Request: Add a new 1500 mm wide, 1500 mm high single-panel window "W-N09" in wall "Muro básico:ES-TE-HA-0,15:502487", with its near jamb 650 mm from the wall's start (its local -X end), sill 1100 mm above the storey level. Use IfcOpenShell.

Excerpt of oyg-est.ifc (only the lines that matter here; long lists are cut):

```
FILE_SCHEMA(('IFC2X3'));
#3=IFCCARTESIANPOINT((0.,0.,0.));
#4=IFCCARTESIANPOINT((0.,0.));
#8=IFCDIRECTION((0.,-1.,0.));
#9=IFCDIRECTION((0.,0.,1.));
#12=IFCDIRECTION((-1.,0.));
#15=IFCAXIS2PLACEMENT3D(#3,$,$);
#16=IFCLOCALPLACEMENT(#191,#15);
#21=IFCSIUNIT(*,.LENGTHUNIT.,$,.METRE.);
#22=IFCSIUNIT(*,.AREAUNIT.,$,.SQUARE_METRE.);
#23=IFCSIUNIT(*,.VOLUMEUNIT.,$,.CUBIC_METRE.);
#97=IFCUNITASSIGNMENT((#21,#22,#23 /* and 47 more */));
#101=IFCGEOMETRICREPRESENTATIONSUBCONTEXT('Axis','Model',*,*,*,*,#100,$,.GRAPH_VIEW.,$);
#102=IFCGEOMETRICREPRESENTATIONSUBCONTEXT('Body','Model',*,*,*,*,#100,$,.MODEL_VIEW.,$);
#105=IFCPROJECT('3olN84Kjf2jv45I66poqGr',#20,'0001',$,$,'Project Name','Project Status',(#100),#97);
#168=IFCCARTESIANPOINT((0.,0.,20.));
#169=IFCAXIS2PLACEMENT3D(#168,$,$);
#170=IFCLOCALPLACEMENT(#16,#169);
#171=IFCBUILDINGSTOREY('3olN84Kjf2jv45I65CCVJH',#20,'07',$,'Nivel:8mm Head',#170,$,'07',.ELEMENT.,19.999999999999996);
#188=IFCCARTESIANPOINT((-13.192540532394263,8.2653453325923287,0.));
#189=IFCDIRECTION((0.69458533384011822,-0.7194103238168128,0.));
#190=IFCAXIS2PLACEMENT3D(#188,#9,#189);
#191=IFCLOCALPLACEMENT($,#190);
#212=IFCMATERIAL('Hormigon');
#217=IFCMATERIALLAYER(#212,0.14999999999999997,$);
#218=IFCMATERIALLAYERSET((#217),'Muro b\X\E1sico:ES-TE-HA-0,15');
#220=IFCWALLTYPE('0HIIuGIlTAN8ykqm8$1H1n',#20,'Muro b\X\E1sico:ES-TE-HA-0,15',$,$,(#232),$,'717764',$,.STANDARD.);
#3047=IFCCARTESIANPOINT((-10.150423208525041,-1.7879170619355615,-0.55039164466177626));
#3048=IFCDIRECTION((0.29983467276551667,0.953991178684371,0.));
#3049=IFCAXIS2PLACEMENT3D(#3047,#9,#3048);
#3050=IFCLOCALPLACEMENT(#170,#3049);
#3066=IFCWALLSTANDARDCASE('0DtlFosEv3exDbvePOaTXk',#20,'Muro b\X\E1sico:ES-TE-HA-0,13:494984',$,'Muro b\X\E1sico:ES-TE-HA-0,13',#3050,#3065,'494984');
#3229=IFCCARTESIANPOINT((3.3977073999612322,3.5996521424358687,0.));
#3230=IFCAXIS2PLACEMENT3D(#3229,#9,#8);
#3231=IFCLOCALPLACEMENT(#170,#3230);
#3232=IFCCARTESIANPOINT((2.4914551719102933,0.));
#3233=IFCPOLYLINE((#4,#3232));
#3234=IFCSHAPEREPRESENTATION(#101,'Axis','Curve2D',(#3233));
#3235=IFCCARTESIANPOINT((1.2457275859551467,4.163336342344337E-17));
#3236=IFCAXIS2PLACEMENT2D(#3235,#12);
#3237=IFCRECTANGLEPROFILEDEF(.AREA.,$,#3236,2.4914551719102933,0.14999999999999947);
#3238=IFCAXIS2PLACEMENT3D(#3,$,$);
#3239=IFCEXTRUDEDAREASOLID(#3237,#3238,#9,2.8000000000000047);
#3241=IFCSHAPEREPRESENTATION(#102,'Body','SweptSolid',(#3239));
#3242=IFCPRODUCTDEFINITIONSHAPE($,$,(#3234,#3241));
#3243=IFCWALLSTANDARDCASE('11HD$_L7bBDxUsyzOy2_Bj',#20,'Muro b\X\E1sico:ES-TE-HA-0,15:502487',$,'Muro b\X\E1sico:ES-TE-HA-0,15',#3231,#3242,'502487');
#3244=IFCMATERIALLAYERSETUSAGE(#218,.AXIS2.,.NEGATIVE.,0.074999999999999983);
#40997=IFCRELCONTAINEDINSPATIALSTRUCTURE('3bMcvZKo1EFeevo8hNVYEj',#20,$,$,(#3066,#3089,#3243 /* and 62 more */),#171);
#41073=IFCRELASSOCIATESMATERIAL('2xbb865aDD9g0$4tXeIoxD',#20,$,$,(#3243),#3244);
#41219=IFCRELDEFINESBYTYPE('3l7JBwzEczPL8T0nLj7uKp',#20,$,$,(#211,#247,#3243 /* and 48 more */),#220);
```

```python
import numpy as np
import ifcopenshell
import ifcopenshell.api.feature
import ifcopenshell.api.geometry
import ifcopenshell.api.root
import ifcopenshell.api.spatial
import ifcopenshell.api.type
import ifcopenshell.geom
import ifcopenshell.util.element
import ifcopenshell.util.placement
import ifcopenshell.util.representation
import ifcopenshell.util.shape
import ifcopenshell.util.unit

model = ifcopenshell.open("oyg-est.ifc")
unit_scale = ifcopenshell.util.unit.calculate_unit_scale(model)
settings = ifcopenshell.geom.settings()


def volume(element):
    """Net volume in cubic metres, openings subtracted."""
    shape = ifcopenshell.geom.create_shape(settings, element)
    return ifcopenshell.util.shape.get_volume(shape.geometry)


wall = model.by_guid("11HD$_L7bBDxUsyzOy2_Bj")
storey = ifcopenshell.util.element.get_container(wall, ifc_class="IfcBuildingStorey")
context = ifcopenshell.util.representation.get_context(model, "Model", "Body", "MODEL_VIEW")
before = volume(wall)

width, height, from_end, sill = 1.5, 1.5, 0.65, 1.1  # metres

# The wall runs along its own X axis, and the end named is its -X end.
wall_shape = ifcopenshell.geom.create_shape(settings, wall)
x, y, z = ifcopenshell.util.shape.get_vertices(wall_shape.geometry).T
start = x.min() + from_end
face, thickness = float(y.min()), float(y.max() - y.min())
wall_matrix = ifcopenshell.util.placement.get_local_placement(wall.ObjectPlacement)
level = ifcopenshell.util.placement.get_local_placement(storey.ObjectPlacement)[2, 3]


def in_wall(x, y):
    """Placement at x, y metres in the wall's axes, at sill height."""
    matrix = wall_matrix.copy()
    matrix[:, 3] = wall_matrix @ np.array([x / unit_scale, y / unit_scale, 0.0, 1.0])
    matrix[2, 3] = level + sill / unit_scale
    return matrix


# Opening: a box that overshoots both wall faces by 50 mm.
opening = ifcopenshell.api.root.create_entity(model, ifc_class="IfcOpeningElement")
box = ifcopenshell.api.geometry.add_wall_representation(
    model, context=context, length=width, height=height, thickness=thickness + 0.1
)
ifcopenshell.api.geometry.assign_representation(model, product=opening, representation=box)
ifcopenshell.api.geometry.edit_object_placement(model, product=opening, matrix=in_wall(start, face - 0.05), is_si=False)
ifcopenshell.api.feature.add_feature(model, feature=opening, element=wall)

window = ifcopenshell.api.root.create_entity(model, ifc_class="IfcWindow", name="W-N09")
window.OverallWidth, window.OverallHeight = width / unit_scale, height / unit_scale
body = ifcopenshell.api.geometry.add_window_representation(
    model,
    context=context,
    overall_width=window.OverallWidth,
    overall_height=window.OverallHeight,
    partition_type="SINGLE_PANEL",
)
ifcopenshell.api.geometry.assign_representation(model, product=window, representation=body)
ifcopenshell.api.spatial.assign_container(model, products=[window], relating_structure=storey)
fills = ifcopenshell.api.feature.add_filling(model, opening=opening, element=window)
fills.OwnerHistory = window.OwnerHistory  # required in IFC2X3

# IFC2X3 keeps the operation on the window style.
style = ifcopenshell.api.root.create_entity(model, ifc_class="IfcWindowStyle", name="W-N09")
style.OperationType, style.ConstructionType = "SINGLE_PANEL", "NOTDEFINED"
style.ParameterTakesPrecedence = style.Sizeable = False
ifcopenshell.api.type.assign_type(model, related_objects=[window], relating_type=style)

# Centre the window in the wall's thickness.
ifcopenshell.api.geometry.edit_object_placement(model, product=window, matrix=in_wall(start, face), is_si=False)
window_shape = ifcopenshell.geom.create_shape(settings, window)
depth = ifcopenshell.util.shape.get_vertices(window_shape.geometry)[:, 1]
offset = face + thickness / 2 - (depth.min() + depth.max()) / 2
ifcopenshell.api.geometry.edit_object_placement(model, product=window, matrix=in_wall(start, offset), is_si=False)

after = volume(wall)

print(f"wall volume {before:.3f} -> {after:.3f} m3")

model.write("oyg-est-out.ifc")
```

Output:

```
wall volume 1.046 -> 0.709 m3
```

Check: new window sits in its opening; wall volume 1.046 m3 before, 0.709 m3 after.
